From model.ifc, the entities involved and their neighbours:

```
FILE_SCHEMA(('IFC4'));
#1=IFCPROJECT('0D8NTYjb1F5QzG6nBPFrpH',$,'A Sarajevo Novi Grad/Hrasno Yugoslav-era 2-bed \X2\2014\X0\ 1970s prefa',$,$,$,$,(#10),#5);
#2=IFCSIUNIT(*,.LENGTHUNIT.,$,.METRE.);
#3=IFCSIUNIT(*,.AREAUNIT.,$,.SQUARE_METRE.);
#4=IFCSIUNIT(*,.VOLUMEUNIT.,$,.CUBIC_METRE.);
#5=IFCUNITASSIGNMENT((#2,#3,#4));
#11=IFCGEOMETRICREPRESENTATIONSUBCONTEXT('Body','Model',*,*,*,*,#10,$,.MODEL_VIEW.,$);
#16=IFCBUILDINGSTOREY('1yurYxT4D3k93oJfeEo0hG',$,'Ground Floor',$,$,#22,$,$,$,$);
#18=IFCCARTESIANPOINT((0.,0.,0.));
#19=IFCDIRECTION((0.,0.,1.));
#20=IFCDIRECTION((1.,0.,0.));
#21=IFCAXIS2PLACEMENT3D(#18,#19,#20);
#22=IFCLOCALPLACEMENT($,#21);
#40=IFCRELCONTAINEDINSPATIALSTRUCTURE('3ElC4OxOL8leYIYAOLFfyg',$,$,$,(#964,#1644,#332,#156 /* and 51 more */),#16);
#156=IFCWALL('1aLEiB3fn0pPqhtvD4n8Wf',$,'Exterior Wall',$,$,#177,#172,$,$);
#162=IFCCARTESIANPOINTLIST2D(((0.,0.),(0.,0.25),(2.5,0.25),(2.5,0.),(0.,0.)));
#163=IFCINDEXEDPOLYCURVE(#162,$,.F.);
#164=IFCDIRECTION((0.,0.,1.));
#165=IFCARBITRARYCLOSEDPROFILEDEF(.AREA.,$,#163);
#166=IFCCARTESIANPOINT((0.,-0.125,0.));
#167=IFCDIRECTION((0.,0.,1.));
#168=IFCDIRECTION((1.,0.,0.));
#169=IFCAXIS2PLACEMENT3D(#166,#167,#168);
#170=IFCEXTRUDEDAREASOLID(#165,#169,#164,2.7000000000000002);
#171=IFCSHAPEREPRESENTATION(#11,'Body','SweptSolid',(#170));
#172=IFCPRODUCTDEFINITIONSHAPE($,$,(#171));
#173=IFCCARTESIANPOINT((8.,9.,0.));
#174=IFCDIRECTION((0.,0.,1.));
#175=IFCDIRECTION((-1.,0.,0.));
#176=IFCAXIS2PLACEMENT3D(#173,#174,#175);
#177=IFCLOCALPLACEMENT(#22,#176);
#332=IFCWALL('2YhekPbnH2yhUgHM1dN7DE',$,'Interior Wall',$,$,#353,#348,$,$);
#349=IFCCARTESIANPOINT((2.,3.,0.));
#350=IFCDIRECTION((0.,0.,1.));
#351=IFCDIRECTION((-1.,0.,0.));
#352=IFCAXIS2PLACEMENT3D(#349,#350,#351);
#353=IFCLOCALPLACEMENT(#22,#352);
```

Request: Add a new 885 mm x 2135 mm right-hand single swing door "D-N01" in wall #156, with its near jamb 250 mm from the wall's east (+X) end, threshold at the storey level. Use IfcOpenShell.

```python
import numpy as np
import ifcopenshell
import ifcopenshell.api.feature
import ifcopenshell.api.geometry
import ifcopenshell.api.root
import ifcopenshell.api.spatial
import ifcopenshell.geom
import ifcopenshell.util.element
import ifcopenshell.util.placement
import ifcopenshell.util.representation
import ifcopenshell.util.shape
import ifcopenshell.util.unit

model = ifcopenshell.open("model.ifc")
unit_scale = ifcopenshell.util.unit.calculate_unit_scale(model)
settings = ifcopenshell.geom.settings()


def volume(element):
    """Net volume in cubic metres, openings subtracted."""
    shape = ifcopenshell.geom.create_shape(settings, element)
    return ifcopenshell.util.shape.get_volume(shape.geometry)


wall = model.by_guid("1aLEiB3fn0pPqhtvD4n8Wf")
storey = ifcopenshell.util.element.get_container(wall, ifc_class="IfcBuildingStorey")
context = ifcopenshell.util.representation.get_context(model, "Model", "Body", "MODEL_VIEW")
before = volume(wall)

width, height, from_end, sill = 0.885, 2.135, 0.25, 0.0  # metres

# The wall runs along its own X axis, and the end named is its -X end.
wall_shape = ifcopenshell.geom.create_shape(settings, wall)
x, y, z = ifcopenshell.util.shape.get_vertices(wall_shape.geometry).T
start = x.min() + from_end
face, thickness = float(y.min()), float(y.max() - y.min())
wall_matrix = ifcopenshell.util.placement.get_local_placement(wall.ObjectPlacement)
level = ifcopenshell.util.placement.get_local_placement(storey.ObjectPlacement)[2, 3]


def in_wall(x, y):
    """Placement at x, y metres in the wall's axes, at sill height."""
    matrix = wall_matrix.copy()
    matrix[:, 3] = wall_matrix @ np.array([x / unit_scale, y / unit_scale, 0.0, 1.0])
    matrix[2, 3] = level + sill / unit_scale
    return matrix


# Opening: a box that overshoots both wall faces by 50 mm.
opening = ifcopenshell.api.root.create_entity(model, ifc_class="IfcOpeningElement", predefined_type="OPENING")
box = ifcopenshell.api.geometry.add_wall_representation(
    model, context=context, length=width, height=height, thickness=thickness + 0.1
)
ifcopenshell.api.geometry.assign_representation(model, product=opening, representation=box)
ifcopenshell.api.geometry.edit_object_placement(model, product=opening, matrix=in_wall(start, face - 0.05), is_si=False)
ifcopenshell.api.feature.add_feature(model, feature=opening, element=wall)

door = ifcopenshell.api.root.create_entity(model, ifc_class="IfcDoor", name="D-N01", predefined_type="DOOR")
door.OverallWidth, door.OverallHeight = width / unit_scale, height / unit_scale
door.OperationType = "SINGLE_SWING_RIGHT"
body = ifcopenshell.api.geometry.add_door_representation(
    model,
    context=context,
    overall_width=door.OverallWidth,
    overall_height=door.OverallHeight,
    operation_type="SINGLE_SWING_RIGHT",
    lining_properties={"LiningDepth": thickness / unit_scale, "ThresholdDepth": thickness / unit_scale},
)
ifcopenshell.api.geometry.assign_representation(model, product=door, representation=body)
ifcopenshell.api.spatial.assign_container(model, products=[door], relating_structure=storey)
ifcopenshell.api.feature.add_filling(model, opening=opening, element=door)

# The lining spans the wall, so the door starts at the wall face.
ifcopenshell.api.geometry.edit_object_placement(model, product=door, matrix=in_wall(start, face), is_si=False)

after = volume(wall)

print(f"wall volume {before:.3f} -> {after:.3f} m3")

model.write("model_v2.ifc")
```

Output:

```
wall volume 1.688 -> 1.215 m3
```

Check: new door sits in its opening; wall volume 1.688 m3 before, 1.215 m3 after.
